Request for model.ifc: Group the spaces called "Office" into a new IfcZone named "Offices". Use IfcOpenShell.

First a look at what the model holds.

```python
import ifcopenshell

model = ifcopenshell.open("model.ifc")
print(model.schema)
seen = {}
for space in model.by_type("IfcSpace"):
    seen[space.LongName] = seen.get(space.LongName, 0) + 1
for name, count in sorted(seen.items(), key=str):
    print(count, "x", name)
print("zones:", [z.Name for z in model.by_type("IfcZone")][:20])
```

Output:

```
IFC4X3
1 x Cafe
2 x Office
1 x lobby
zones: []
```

```python
import ifcopenshell
import ifcopenshell.api.group
import ifcopenshell.api.root

model = ifcopenshell.open("model.ifc")

names = {"Office"}
spaces = [s for s in model.by_type("IfcSpace") if s.LongName in names]

zone = ifcopenshell.api.root.create_entity(model, ifc_class="IfcZone", name="Offices")
ifcopenshell.api.group.assign_group(model, products=spaces, group=zone)
print(len(spaces), "spaces in", zone.Name)

model.write("model_edited.ifc")
```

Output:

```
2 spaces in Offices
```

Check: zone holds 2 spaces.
